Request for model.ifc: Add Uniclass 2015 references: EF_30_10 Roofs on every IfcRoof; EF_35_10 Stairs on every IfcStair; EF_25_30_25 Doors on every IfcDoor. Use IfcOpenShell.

First a look at what the model holds.

```python
import ifcopenshell

model = ifcopenshell.open("model.ifc")
print(model.schema)
print("classifications:", [c.Name for c in model.by_type("IfcClassification")])
for ifc_class in ("IfcDoor", "IfcRoof", "IfcStair", "IfcWall", "IfcWindow"):
    print(ifc_class, len(model.by_type(ifc_class)))
```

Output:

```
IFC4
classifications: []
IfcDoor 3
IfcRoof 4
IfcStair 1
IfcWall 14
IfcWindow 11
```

```python
import ifcopenshell
import ifcopenshell.api.classification

model = ifcopenshell.open("model.ifc")

system = ifcopenshell.api.classification.add_classification(model, classification="Uniclass 2015")

codes = {
    "IfcRoof": ("EF_30_10", "Roofs"),
    "IfcStair": ("EF_35_10", "Stairs"),
    "IfcDoor": ("EF_25_30_25", "Doors"),
}
for ifc_class, (code, name) in codes.items():
    products = model.by_type(ifc_class)
    ifcopenshell.api.classification.add_reference(
        model, products=products, classification=system, identification=code, name=name
    )
    print(code, len(products))

model.write("model_updated.ifc")
```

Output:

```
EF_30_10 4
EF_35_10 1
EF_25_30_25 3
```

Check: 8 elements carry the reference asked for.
